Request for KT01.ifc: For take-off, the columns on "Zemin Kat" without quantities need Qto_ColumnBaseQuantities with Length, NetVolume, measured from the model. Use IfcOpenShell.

First a look at what the model holds.

```python
import ifcopenshell
import ifcopenshell.util.element
import ifcopenshell.util.unit

model = ifcopenshell.open("KT01.ifc")
print(model.schema)
for unit_type in ("LENGTHUNIT", "AREAUNIT", "VOLUMEUNIT"):
    print(unit_type, ifcopenshell.util.unit.calculate_unit_scale(model, unit_type))
storey = next(s for s in model.by_type("IfcBuildingStorey") if s.Name == "Zemin Kat")
columns = [e for e in ifcopenshell.util.element.get_decomposition(storey) if e.is_a("IfcColumn")]
for e in sorted(columns, key=lambda e: e.id()):
    print(e.id(), e.is_a(), e.Name, list(ifcopenshell.util.element.get_psets(e, qtos_only=True)), sep=" | ")
```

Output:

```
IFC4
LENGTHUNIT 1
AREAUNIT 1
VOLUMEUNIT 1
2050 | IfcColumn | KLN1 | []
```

```python
import ifcopenshell
import ifcopenshell.api.pset
import ifcopenshell.geom
import ifcopenshell.util.element
import ifcopenshell.util.shape
import ifcopenshell.util.unit

model = ifcopenshell.open("KT01.ifc")
unit_scale = ifcopenshell.util.unit.calculate_unit_scale(model)
volume_scale = ifcopenshell.util.unit.calculate_unit_scale(model, "VOLUMEUNIT")
settings = ifcopenshell.geom.settings()

storey = next(s for s in model.by_type("IfcBuildingStorey") if s.Name == "Zemin Kat")
columns = [e for e in ifcopenshell.util.element.get_decomposition(storey) if e.is_a("IfcColumn")]

for e in sorted(columns, key=lambda e: e.id()):
    if ifcopenshell.util.element.get_psets(e, qtos_only=True, should_inherit=False):
        continue
    # Geometry comes back in metres, in the element's own axes.
    shape = ifcopenshell.geom.create_shape(settings, e)
    values = {
        "Length": ifcopenshell.util.shape.get_z(shape.geometry) / unit_scale,
        "NetVolume": ifcopenshell.util.shape.get_volume(shape.geometry) / volume_scale,
    }
    qto = ifcopenshell.api.pset.add_qto(model, product=e, name="Qto_ColumnBaseQuantities")
    ifcopenshell.api.pset.edit_qto(model, qto=qto, properties=values)
    print(e.id(), {k: round(v, 3) for k, v in values.items()})

model.write("KT01_v2.ifc")
```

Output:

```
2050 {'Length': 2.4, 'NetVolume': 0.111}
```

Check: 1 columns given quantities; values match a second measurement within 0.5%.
